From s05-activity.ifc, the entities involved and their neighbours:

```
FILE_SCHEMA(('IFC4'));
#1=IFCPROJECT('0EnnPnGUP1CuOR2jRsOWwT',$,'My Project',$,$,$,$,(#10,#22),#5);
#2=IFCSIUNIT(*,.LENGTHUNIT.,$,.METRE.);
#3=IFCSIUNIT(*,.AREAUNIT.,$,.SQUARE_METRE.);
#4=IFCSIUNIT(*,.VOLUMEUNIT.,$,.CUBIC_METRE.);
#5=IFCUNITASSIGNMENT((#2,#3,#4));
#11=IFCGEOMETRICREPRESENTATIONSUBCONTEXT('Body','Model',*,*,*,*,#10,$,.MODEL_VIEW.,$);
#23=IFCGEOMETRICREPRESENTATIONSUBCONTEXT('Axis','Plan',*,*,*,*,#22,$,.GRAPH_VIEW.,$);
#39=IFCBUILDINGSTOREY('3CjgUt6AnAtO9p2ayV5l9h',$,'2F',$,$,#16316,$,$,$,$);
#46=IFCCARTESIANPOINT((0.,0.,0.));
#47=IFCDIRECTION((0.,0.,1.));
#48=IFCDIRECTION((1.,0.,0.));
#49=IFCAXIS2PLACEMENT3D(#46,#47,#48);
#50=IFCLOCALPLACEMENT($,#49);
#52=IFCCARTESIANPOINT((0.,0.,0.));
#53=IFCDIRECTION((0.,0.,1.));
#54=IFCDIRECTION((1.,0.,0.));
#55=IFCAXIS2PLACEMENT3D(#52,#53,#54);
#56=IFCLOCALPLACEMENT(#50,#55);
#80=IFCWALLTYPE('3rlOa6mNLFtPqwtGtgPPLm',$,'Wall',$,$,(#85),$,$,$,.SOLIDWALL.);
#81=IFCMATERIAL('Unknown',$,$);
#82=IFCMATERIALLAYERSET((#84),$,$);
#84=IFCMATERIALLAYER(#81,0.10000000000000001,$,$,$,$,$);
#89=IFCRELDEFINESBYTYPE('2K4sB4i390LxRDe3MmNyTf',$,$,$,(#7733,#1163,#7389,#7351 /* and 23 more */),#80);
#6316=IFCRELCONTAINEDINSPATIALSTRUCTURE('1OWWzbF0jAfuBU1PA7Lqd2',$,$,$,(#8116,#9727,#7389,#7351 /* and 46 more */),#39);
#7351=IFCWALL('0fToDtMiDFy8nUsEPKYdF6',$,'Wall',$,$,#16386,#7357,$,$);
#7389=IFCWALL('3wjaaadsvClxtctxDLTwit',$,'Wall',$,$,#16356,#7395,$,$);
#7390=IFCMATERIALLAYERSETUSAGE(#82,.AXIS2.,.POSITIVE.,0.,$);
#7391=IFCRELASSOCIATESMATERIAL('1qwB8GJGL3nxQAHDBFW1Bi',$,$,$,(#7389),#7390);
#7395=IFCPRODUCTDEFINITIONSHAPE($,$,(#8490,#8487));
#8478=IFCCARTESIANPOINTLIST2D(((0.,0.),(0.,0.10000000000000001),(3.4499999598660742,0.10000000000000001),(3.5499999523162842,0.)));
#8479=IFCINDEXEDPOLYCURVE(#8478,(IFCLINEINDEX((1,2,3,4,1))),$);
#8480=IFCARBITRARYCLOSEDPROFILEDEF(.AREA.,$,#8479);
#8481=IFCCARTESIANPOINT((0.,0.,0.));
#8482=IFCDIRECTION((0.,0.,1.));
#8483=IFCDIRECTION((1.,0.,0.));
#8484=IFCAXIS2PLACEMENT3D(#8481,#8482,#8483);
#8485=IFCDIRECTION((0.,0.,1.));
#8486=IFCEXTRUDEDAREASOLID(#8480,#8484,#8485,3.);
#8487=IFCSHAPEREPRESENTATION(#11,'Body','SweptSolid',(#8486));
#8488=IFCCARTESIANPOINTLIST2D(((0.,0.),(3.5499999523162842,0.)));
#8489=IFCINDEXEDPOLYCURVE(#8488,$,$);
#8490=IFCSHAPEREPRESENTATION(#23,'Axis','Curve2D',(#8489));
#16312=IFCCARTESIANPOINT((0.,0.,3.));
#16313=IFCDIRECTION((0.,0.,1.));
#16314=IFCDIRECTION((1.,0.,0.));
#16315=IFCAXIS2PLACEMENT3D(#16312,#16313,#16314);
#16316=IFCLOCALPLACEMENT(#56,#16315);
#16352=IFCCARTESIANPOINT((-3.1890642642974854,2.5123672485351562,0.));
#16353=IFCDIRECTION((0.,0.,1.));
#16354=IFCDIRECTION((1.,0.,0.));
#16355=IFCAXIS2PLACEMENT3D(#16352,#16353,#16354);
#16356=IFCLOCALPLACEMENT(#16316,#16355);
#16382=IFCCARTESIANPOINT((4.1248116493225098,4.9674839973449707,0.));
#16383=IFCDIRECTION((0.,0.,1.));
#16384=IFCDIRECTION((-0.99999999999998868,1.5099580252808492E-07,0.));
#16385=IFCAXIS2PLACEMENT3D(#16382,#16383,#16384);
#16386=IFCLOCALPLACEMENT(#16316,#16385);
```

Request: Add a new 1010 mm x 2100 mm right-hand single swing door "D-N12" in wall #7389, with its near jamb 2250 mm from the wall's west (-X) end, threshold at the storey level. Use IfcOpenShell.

```python
import numpy as np
import ifcopenshell
import ifcopenshell.api.feature
import ifcopenshell.api.geometry
import ifcopenshell.api.root
import ifcopenshell.api.spatial
import ifcopenshell.geom
import ifcopenshell.util.element
import ifcopenshell.util.placement
import ifcopenshell.util.representation
import ifcopenshell.util.shape
import ifcopenshell.util.unit

model = ifcopenshell.open("s05-activity.ifc")
unit_scale = ifcopenshell.util.unit.calculate_unit_scale(model)
settings = ifcopenshell.geom.settings()


def volume(element):
    """Net volume in cubic metres, openings subtracted."""
    shape = ifcopenshell.geom.create_shape(settings, element)
    return ifcopenshell.util.shape.get_volume(shape.geometry)


wall = model.by_guid("3wjaaadsvClxtctxDLTwit")
storey = ifcopenshell.util.element.get_container(wall, ifc_class="IfcBuildingStorey")
context = ifcopenshell.util.representation.get_context(model, "Model", "Body", "MODEL_VIEW")
before = volume(wall)

width, height, from_end, sill = 1.01, 2.1, 2.25, 0.0  # metres

# The wall runs along its own X axis, and the end named is its -X end.
wall_shape = ifcopenshell.geom.create_shape(settings, wall)
x, y, z = ifcopenshell.util.shape.get_vertices(wall_shape.geometry).T
start = x.min() + from_end
face, thickness = float(y.min()), float(y.max() - y.min())
wall_matrix = ifcopenshell.util.placement.get_local_placement(wall.ObjectPlacement)
level = ifcopenshell.util.placement.get_local_placement(storey.ObjectPlacement)[2, 3]


def in_wall(x, y):
    """Placement at x, y metres in the wall's axes, at sill height."""
    matrix = wall_matrix.copy()
    matrix[:, 3] = wall_matrix @ np.array([x / unit_scale, y / unit_scale, 0.0, 1.0])
    matrix[2, 3] = level + sill / unit_scale
    return matrix


# Opening: a box that overshoots both wall faces by 50 mm.
opening = ifcopenshell.api.root.create_entity(model, ifc_class="IfcOpeningElement", predefined_type="OPENING")
box = ifcopenshell.api.geometry.add_wall_representation(
    model, context=context, length=width, height=height, thickness=thickness + 0.1
)
ifcopenshell.api.geometry.assign_representation(model, product=opening, representation=box)
ifcopenshell.api.geometry.edit_object_placement(model, product=opening, matrix=in_wall(start, face - 0.05), is_si=False)
ifcopenshell.api.feature.add_feature(model, feature=opening, element=wall)

door = ifcopenshell.api.root.create_entity(model, ifc_class="IfcDoor", name="D-N12", predefined_type="DOOR")
door.OverallWidth, door.OverallHeight = width / unit_scale, height / unit_scale
door.OperationType = "SINGLE_SWING_RIGHT"
body = ifcopenshell.api.geometry.add_door_representation(
    model,
    context=context,
    overall_width=door.OverallWidth,
    overall_height=door.OverallHeight,
    operation_type="SINGLE_SWING_RIGHT",
    lining_properties={"LiningDepth": thickness / unit_scale, "ThresholdDepth": thickness / unit_scale},
)
ifcopenshell.api.geometry.assign_representation(model, product=door, representation=body)
ifcopenshell.api.spatial.assign_container(model, products=[door], relating_structure=storey)
ifcopenshell.api.feature.add_filling(model, opening=opening, element=door)

# The lining spans the wall, so the door starts at the wall face.
ifcopenshell.api.geometry.edit_object_placement(model, product=door, matrix=in_wall(start, face), is_si=False)

after = volume(wall)

print(f"wall volume {before:.3f} -> {after:.3f} m3")

model.write("s05-activity_edited.ifc")
```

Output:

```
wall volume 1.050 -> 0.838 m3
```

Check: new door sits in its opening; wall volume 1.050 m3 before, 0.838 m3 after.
